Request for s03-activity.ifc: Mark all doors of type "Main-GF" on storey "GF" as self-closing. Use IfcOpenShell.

First a look at what the model holds.

```python
import ifcopenshell
import ifcopenshell.util.element

model = ifcopenshell.open("s03-activity.ifc")
print(model.schema)
storey = next(s for s in model.by_type("IfcBuildingStorey") if s.Name == "GF")
doors = [e for e in ifcopenshell.util.element.get_decomposition(storey) if e.is_a("IfcDoor")]
seen = {}
for e in doors:
    element_type = ifcopenshell.util.element.get_type(e)
    key = (element_type.Name if element_type != e and element_type else None, ifcopenshell.util.element.get_pset(e, "Pset_DoorCommon", "SelfClosing"))
    seen[key] = seen.get(key, 0) + 1
for (name, value), count in sorted(seen.items(), key=str):
    print(count, "x", name, "|", value)
```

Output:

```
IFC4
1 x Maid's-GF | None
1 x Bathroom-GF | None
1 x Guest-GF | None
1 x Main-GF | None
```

```python
import ifcopenshell
import ifcopenshell.api.pset
import ifcopenshell.util.element

model = ifcopenshell.open("s03-activity.ifc")

storey = next(s for s in model.by_type("IfcBuildingStorey") if s.Name == "GF")
doors = [e for e in ifcopenshell.util.element.get_decomposition(storey) if e.is_a("IfcDoor")]

count = 0
for e in doors:
    element_type = ifcopenshell.util.element.get_type(e)
    if element_type in (None, e) or element_type.Name != "Main-GF":
        continue
    # add_pset returns the element's existing set when there is one.
    pset = ifcopenshell.api.pset.add_pset(model, product=e, name="Pset_DoorCommon")
    ifcopenshell.api.pset.edit_pset(model, pset=pset, properties={"SelfClosing": True})
    count += 1

print(count, "doors updated")

model.write("s03-activity-out.ifc")
```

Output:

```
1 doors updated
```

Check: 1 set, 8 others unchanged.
